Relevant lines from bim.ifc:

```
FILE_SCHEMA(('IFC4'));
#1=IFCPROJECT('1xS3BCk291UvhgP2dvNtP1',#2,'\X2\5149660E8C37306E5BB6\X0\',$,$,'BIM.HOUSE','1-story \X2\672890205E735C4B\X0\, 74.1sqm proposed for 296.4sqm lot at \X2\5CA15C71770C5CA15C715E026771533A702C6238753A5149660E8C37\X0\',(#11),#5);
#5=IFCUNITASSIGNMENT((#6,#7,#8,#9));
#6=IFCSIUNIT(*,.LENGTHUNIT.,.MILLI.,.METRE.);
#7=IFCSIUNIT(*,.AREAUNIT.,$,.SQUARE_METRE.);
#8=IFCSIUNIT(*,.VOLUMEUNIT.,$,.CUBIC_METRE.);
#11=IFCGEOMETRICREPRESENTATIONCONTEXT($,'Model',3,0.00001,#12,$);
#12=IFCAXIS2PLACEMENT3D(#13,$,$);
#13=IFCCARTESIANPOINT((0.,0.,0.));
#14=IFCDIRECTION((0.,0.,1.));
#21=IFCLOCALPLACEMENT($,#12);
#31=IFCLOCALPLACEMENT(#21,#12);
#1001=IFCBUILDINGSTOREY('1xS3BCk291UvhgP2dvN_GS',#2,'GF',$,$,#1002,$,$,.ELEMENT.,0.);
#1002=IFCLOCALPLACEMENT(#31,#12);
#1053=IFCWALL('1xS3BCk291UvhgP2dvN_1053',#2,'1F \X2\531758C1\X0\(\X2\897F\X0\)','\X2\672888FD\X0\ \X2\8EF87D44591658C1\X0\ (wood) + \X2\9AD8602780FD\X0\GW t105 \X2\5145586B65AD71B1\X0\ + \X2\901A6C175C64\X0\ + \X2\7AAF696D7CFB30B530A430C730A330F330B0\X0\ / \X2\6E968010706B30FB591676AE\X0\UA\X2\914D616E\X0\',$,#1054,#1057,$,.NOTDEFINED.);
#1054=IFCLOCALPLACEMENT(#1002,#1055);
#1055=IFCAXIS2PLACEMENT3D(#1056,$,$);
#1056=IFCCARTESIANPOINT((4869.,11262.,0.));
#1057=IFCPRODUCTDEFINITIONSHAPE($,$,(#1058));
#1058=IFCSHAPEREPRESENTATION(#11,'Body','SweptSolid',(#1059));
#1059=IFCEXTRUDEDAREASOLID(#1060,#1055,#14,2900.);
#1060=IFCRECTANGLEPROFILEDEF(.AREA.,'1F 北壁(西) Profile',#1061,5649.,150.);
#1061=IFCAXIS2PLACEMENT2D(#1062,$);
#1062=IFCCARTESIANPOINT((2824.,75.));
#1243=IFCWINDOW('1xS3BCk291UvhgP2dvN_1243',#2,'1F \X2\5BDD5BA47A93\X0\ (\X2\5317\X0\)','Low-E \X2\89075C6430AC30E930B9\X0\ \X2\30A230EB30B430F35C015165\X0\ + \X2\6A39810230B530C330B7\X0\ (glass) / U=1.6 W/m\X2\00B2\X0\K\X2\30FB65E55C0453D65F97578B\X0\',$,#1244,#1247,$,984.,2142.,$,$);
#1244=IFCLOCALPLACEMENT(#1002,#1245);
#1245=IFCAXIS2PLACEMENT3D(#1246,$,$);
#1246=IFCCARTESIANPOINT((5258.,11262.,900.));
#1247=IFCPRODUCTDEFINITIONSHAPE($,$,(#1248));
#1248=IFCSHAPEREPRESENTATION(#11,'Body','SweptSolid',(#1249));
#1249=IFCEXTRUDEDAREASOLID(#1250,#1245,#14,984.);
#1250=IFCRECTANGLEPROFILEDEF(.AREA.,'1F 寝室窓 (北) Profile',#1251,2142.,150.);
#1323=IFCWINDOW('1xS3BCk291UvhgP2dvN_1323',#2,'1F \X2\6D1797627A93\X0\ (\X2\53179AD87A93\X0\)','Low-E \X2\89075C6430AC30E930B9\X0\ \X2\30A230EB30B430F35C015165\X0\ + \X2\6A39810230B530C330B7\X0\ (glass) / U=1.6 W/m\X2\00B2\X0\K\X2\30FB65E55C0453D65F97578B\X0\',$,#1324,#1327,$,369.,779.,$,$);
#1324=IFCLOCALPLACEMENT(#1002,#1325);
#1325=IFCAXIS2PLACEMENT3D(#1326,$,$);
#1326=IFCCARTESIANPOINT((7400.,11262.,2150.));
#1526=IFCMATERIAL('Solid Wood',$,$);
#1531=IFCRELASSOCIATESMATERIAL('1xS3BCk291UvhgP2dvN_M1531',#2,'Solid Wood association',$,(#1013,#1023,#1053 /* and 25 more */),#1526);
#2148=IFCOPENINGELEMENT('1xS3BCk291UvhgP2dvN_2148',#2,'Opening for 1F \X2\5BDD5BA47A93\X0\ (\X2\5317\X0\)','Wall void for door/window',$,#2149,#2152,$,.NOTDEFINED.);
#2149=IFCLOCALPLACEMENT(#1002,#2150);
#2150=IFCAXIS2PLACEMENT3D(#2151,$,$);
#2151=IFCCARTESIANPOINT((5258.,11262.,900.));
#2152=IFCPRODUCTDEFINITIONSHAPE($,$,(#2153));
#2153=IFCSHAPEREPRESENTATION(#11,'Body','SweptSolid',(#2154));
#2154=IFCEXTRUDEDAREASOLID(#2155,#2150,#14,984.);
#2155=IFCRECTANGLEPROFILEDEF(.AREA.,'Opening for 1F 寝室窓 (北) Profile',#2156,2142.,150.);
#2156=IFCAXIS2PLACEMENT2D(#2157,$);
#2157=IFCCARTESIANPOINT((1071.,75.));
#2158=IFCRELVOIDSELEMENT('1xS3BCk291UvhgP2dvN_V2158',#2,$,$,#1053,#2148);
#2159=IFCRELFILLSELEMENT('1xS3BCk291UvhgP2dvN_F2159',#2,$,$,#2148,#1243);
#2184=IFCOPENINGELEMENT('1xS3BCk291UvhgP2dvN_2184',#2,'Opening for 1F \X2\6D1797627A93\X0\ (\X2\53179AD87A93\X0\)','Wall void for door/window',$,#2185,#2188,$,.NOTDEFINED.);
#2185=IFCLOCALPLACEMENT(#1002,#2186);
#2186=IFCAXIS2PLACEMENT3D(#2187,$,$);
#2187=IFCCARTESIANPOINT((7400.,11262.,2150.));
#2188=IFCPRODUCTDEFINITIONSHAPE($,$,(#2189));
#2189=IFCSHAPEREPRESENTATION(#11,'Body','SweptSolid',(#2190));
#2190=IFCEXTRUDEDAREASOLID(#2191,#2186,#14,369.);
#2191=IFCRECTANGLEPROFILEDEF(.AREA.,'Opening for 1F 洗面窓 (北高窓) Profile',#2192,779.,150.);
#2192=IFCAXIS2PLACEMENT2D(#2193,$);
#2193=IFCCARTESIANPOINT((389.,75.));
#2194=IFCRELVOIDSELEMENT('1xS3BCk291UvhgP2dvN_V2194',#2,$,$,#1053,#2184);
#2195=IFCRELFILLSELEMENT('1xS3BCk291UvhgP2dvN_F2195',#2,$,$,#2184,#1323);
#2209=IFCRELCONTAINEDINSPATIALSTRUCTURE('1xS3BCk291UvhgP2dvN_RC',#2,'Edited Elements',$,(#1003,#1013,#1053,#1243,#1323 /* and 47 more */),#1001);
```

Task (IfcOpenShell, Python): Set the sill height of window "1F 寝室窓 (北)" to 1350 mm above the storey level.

```python
import numpy as np
import ifcopenshell
import ifcopenshell.api.geometry
import ifcopenshell.geom
import ifcopenshell.util.element
import ifcopenshell.util.placement
import ifcopenshell.util.shape
import ifcopenshell.util.unit

model = ifcopenshell.open("bim.ifc")
unit_scale = ifcopenshell.util.unit.calculate_unit_scale(model)

window = model.by_guid("1xS3BCk291UvhgP2dvN_1243")
opening = window.FillsVoids[0].RelatingOpeningElement
storey = ifcopenshell.util.element.get_container(window, ifc_class="IfcBuildingStorey")
level = ifcopenshell.util.placement.get_local_placement(storey.ObjectPlacement)[2, 3]

# The opening's origin need not be at the sill, so measure its lowest point.
shape = ifcopenshell.geom.create_shape(ifcopenshell.geom.settings(), opening)
bottom = ifcopenshell.util.shape.get_shape_bottom_elevation(shape, shape.geometry) / unit_scale
dz = level + 1.35 / unit_scale - bottom

shift = np.array([0.0, 0.0, dz])
# The window is not placed relative to its opening, so move both.
for product in (opening, window):
    matrix = ifcopenshell.util.placement.get_local_placement(product.ObjectPlacement)
    matrix[:3, 3] += shift
    ifcopenshell.api.geometry.edit_object_placement(model, product=product, matrix=matrix, is_si=False)

print(f"moved by {dz * unit_scale:+.3f} m")

model.write("bim_updated.ifc")
```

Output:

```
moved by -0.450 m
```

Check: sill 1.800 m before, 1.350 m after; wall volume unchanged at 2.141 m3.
